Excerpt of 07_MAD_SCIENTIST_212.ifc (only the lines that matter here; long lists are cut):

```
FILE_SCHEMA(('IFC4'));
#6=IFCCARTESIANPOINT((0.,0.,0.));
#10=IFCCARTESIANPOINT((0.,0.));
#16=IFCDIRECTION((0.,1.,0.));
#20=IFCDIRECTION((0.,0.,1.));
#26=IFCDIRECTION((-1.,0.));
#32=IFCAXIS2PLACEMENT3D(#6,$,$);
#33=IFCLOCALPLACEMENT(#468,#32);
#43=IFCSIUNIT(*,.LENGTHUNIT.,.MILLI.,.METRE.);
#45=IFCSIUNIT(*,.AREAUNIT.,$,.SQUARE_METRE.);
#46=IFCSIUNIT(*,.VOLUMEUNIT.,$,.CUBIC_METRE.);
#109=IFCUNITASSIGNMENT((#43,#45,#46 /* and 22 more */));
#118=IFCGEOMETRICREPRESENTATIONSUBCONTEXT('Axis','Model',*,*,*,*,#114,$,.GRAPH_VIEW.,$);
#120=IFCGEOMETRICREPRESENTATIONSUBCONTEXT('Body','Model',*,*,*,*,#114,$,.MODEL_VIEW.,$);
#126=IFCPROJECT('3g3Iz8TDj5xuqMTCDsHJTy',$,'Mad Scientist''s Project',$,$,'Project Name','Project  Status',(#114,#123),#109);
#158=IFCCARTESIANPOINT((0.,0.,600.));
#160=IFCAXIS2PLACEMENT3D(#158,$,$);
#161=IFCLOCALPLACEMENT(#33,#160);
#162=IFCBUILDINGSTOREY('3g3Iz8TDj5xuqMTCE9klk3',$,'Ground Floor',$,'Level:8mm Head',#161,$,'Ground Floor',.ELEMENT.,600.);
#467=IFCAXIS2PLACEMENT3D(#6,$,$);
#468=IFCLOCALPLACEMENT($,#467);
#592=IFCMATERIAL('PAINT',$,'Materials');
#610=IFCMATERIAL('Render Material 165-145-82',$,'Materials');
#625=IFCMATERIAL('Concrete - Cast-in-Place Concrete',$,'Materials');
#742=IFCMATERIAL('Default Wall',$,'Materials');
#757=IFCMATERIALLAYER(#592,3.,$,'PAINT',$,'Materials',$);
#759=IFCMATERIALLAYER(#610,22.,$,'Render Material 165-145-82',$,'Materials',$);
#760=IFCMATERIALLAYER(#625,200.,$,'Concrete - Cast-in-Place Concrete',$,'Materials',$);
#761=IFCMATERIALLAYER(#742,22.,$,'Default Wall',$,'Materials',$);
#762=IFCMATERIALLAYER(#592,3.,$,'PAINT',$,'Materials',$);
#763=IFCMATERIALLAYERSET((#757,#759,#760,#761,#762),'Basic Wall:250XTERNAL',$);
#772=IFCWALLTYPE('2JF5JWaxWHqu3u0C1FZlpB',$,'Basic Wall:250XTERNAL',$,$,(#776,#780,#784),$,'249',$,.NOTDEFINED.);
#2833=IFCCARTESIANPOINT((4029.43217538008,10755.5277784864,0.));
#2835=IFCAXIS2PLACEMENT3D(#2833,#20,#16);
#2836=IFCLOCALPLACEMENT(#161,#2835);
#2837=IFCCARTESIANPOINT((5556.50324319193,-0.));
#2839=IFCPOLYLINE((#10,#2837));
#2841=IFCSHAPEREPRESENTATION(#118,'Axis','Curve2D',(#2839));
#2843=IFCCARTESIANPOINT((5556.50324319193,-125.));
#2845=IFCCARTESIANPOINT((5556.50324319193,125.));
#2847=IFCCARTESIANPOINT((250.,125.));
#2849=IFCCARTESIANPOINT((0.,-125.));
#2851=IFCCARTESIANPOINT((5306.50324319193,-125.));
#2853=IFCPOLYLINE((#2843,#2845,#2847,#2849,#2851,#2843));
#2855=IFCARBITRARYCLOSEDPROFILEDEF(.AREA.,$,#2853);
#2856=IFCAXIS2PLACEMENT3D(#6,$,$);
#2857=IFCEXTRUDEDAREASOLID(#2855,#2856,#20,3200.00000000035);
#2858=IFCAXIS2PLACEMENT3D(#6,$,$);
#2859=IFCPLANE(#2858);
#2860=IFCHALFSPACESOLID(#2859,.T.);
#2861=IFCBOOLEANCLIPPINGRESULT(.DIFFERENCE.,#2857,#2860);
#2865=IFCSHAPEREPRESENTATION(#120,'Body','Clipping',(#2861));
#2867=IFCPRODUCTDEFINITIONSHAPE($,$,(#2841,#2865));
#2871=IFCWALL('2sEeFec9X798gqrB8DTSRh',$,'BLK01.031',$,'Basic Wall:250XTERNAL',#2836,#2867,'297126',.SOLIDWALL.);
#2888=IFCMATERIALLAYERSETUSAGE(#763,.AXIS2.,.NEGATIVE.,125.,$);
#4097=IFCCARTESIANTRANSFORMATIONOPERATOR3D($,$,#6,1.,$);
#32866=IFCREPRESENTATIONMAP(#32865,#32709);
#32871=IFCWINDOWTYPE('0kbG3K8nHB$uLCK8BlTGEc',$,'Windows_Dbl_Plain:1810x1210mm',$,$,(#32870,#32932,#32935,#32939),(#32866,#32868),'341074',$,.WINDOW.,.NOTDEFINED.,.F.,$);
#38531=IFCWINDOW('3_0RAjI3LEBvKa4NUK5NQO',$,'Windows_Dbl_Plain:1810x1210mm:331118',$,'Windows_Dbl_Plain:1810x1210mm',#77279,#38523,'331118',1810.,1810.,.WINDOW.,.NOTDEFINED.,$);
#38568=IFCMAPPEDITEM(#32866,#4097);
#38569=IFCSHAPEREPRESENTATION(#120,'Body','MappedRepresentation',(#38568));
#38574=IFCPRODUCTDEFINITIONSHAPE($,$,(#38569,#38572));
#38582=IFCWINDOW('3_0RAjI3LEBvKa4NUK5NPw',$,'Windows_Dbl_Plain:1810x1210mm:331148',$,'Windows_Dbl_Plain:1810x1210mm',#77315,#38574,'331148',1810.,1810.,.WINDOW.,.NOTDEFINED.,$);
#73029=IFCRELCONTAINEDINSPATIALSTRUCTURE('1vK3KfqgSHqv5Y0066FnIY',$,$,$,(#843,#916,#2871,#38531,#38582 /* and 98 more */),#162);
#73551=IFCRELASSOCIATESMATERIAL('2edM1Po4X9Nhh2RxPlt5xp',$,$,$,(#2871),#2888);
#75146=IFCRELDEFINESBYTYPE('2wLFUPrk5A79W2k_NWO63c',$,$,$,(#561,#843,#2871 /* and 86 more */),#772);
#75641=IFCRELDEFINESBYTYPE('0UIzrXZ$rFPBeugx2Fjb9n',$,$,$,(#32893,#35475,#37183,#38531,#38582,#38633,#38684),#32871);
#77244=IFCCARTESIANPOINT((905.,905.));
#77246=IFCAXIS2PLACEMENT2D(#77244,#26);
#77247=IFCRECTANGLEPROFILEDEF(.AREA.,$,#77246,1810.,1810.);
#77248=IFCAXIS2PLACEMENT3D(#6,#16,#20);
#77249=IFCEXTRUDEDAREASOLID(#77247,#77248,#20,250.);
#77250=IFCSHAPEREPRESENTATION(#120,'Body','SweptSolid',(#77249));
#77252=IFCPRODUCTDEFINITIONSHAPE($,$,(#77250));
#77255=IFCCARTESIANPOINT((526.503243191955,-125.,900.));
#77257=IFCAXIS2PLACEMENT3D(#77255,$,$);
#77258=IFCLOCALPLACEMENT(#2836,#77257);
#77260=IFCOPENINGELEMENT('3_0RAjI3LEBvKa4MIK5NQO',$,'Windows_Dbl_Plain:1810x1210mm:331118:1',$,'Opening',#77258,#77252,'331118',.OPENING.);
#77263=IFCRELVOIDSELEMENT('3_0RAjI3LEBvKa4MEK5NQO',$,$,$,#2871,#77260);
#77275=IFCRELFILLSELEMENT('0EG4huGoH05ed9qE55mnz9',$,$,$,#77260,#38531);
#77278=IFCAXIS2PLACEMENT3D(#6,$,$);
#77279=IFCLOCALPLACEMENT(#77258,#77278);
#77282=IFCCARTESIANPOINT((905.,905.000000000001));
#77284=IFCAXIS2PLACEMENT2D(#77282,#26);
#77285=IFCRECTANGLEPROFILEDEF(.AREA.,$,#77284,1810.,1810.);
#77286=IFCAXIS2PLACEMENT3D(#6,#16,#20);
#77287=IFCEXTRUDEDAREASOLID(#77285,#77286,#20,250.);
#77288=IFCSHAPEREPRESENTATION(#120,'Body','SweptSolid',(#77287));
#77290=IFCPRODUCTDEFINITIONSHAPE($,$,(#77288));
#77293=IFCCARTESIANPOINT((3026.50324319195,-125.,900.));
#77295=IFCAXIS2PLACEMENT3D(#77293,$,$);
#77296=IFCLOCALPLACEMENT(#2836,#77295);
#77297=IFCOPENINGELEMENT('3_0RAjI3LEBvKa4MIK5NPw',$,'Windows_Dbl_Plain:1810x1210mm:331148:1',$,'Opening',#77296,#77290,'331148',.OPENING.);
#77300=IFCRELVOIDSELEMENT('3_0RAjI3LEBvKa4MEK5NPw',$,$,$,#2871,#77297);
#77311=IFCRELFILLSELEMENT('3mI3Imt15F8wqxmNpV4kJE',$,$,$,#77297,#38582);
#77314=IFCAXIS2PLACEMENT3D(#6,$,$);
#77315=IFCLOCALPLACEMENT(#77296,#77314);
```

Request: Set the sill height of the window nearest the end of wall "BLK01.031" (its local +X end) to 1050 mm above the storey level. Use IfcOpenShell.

```python
import numpy as np
import ifcopenshell
import ifcopenshell.api.geometry
import ifcopenshell.geom
import ifcopenshell.util.element
import ifcopenshell.util.placement
import ifcopenshell.util.shape
import ifcopenshell.util.unit

model = ifcopenshell.open("07_MAD_SCIENTIST_212.ifc")
unit_scale = ifcopenshell.util.unit.calculate_unit_scale(model)

window = model.by_id(38582)
opening = window.FillsVoids[0].RelatingOpeningElement
storey = ifcopenshell.util.element.get_container(window, ifc_class="IfcBuildingStorey")
level = ifcopenshell.util.placement.get_local_placement(storey.ObjectPlacement)[2, 3]

# The opening's origin need not be at the sill, so measure its lowest point.
shape = ifcopenshell.geom.create_shape(ifcopenshell.geom.settings(), opening)
bottom = ifcopenshell.util.shape.get_shape_bottom_elevation(shape, shape.geometry) / unit_scale
dz = level + 1050.0 - bottom

shift = np.array([0.0, 0.0, dz])
# The window is placed relative to its opening, so it follows when the opening moves.
matrix = ifcopenshell.util.placement.get_local_placement(opening.ObjectPlacement)
matrix[:3, 3] += shift
ifcopenshell.api.geometry.edit_object_placement(
    model, product=opening, matrix=matrix, is_si=False, should_transform_children=True
)

print(f"moved by {dz * unit_scale:+.3f} m")

model.write("07_MAD_SCIENTIST_212_edited.ifc")
```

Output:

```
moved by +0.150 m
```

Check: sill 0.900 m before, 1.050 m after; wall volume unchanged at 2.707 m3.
